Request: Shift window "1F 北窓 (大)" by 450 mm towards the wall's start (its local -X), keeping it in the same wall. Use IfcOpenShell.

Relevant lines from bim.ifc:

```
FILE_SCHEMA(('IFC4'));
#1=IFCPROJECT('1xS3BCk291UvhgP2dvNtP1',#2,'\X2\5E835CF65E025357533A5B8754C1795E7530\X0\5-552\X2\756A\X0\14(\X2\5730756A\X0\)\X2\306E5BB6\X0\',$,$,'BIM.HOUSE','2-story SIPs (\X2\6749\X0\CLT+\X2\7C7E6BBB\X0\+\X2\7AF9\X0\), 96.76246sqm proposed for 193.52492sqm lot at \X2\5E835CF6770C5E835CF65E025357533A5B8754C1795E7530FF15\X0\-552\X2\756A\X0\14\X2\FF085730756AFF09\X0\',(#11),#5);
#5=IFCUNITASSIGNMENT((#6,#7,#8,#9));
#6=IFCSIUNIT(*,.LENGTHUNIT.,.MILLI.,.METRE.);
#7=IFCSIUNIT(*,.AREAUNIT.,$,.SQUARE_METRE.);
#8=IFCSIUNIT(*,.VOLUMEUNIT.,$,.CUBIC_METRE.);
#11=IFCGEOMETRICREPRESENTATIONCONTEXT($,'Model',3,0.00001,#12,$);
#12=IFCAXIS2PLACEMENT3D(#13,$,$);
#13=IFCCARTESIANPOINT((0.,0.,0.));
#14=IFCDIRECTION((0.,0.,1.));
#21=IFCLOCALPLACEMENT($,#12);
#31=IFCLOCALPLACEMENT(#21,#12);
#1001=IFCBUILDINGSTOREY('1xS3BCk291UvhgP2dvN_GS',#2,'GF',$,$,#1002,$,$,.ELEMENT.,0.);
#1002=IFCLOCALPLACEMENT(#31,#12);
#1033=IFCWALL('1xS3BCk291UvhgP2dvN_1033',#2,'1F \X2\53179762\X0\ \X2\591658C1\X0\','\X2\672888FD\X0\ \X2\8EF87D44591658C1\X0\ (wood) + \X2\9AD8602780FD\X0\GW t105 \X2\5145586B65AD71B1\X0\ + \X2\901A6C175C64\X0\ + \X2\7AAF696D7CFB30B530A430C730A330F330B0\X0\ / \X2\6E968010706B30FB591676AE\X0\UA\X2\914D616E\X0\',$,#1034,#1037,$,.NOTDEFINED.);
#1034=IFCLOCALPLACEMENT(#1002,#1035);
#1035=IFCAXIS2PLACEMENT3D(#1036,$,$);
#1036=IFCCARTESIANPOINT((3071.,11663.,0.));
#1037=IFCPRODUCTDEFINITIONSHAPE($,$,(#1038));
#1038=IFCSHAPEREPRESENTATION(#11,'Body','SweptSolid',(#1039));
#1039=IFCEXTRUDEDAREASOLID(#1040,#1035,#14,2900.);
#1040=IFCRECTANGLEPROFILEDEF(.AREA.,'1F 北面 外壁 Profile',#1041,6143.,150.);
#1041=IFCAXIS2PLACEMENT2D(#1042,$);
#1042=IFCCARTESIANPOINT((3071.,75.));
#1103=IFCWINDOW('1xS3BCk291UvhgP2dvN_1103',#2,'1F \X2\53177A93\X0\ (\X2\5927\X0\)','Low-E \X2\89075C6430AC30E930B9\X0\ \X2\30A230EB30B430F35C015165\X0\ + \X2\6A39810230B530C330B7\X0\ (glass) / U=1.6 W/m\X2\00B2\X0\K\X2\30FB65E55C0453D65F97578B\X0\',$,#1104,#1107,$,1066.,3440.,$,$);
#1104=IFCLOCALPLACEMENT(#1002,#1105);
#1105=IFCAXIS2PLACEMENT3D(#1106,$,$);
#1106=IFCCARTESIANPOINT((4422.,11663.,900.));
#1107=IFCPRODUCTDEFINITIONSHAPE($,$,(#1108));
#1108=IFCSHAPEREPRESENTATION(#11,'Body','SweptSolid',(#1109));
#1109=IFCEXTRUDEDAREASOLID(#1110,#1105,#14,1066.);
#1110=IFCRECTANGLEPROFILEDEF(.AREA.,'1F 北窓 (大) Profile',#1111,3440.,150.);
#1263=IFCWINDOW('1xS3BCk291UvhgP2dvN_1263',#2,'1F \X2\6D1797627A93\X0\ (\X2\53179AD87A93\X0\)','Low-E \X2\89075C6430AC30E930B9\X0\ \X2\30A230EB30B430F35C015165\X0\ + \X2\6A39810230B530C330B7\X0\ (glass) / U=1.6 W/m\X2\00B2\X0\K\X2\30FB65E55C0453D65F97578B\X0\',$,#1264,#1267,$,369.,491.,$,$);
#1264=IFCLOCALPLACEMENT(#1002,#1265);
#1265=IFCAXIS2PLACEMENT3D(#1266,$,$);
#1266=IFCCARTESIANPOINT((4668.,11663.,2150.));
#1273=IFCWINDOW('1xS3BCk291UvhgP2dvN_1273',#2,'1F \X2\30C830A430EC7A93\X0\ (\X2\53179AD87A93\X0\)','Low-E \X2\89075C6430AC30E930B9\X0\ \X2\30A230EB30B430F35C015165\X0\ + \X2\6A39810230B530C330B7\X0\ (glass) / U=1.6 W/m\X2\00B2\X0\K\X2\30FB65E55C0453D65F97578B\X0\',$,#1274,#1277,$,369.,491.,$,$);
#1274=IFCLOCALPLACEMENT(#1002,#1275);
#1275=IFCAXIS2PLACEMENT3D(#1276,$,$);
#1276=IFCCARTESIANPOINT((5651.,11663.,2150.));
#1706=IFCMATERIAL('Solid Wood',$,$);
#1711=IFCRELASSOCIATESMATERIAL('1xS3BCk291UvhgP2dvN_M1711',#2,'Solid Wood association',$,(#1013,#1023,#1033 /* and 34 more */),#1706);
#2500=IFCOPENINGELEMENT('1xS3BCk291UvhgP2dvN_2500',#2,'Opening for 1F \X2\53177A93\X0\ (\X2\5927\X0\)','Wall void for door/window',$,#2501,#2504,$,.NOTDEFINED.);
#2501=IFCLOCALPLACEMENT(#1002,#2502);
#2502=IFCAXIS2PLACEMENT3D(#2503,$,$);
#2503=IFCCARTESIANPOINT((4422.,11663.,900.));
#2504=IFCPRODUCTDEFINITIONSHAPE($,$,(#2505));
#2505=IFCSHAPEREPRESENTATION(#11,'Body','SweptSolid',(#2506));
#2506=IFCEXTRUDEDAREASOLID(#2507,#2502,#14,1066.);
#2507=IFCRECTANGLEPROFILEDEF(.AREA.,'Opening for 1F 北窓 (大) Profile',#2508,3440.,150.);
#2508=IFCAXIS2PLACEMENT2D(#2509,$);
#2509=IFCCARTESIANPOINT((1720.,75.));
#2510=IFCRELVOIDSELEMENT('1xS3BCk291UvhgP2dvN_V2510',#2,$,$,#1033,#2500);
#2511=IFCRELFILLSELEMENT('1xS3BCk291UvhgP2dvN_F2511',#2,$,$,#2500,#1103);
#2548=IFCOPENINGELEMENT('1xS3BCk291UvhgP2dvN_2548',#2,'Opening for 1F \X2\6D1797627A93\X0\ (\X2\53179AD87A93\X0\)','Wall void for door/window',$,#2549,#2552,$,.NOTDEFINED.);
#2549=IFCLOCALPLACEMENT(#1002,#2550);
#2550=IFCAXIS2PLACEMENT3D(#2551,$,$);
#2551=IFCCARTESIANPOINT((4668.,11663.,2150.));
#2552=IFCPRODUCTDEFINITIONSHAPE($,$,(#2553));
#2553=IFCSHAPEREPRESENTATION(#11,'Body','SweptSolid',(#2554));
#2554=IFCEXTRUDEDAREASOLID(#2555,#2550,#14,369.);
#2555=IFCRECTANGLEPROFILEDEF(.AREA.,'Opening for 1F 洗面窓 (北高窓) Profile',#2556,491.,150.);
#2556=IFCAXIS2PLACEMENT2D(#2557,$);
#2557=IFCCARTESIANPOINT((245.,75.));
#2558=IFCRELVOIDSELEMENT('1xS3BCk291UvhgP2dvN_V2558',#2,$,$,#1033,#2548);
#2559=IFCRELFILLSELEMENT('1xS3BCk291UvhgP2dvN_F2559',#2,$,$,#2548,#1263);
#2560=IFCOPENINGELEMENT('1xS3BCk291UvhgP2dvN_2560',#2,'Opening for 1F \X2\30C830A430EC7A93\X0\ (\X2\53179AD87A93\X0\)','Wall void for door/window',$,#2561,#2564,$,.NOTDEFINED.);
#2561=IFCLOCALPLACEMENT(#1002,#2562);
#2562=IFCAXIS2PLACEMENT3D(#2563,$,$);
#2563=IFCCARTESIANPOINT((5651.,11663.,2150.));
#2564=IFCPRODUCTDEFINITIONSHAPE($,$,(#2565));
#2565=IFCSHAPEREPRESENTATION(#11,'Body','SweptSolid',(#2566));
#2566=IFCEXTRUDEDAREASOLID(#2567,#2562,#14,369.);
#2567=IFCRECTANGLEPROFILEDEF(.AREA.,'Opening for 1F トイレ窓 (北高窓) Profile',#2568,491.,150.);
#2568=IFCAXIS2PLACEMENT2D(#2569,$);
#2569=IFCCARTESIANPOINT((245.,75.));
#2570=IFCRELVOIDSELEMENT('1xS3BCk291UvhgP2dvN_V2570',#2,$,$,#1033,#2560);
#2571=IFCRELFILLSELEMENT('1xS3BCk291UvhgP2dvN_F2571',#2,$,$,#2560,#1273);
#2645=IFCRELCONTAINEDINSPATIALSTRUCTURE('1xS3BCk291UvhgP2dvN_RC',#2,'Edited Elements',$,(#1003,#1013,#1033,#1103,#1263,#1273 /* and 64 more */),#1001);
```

```python
import ifcopenshell
import ifcopenshell.api.geometry
import ifcopenshell.util.placement

model = ifcopenshell.open("bim.ifc")

window = model.by_id(1103)
opening = window.FillsVoids[0].RelatingOpeningElement
wall = opening.VoidsElements[0].RelatingBuildingElement

wall_matrix = ifcopenshell.util.placement.get_local_placement(wall.ObjectPlacement)
shift = wall_matrix[:3, 0] * -450.0
before = ifcopenshell.util.placement.get_local_placement(window.ObjectPlacement)[:3, 3].copy()

# The window is not placed relative to its opening, so move both.
for product in (opening, window):
    matrix = ifcopenshell.util.placement.get_local_placement(product.ObjectPlacement)
    matrix[:3, 3] += shift
    ifcopenshell.api.geometry.edit_object_placement(model, product=product, matrix=matrix, is_si=False)

after = ifcopenshell.util.placement.get_local_placement(window.ObjectPlacement)[:3, 3]
print("window moved by", (after - before).round(3) + 0.0)

model.write("bim_rev.ifc")
```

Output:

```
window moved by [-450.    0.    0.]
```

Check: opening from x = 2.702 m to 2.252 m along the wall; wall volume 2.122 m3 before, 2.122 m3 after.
